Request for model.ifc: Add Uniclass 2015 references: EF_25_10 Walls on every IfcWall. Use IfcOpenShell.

First a look at what the model holds.

```python
import ifcopenshell

model = ifcopenshell.open("model.ifc")
print(model.schema)
print("classifications:", [c.Name for c in model.by_type("IfcClassification")])
for ifc_class in ("IfcDoor", "IfcRoof", "IfcStair", "IfcWall", "IfcWindow"):
    print(ifc_class, len(model.by_type(ifc_class)))
```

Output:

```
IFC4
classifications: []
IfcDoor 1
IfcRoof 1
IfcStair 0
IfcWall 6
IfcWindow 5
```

```python
import ifcopenshell
import ifcopenshell.api.classification

model = ifcopenshell.open("model.ifc")

system = ifcopenshell.api.classification.add_classification(model, classification="Uniclass 2015")

codes = {
    "IfcWall": ("EF_25_10", "Walls"),
}
for ifc_class, (code, name) in codes.items():
    products = model.by_type(ifc_class)
    ifcopenshell.api.classification.add_reference(
        model, products=products, classification=system, identification=code, name=name
    )
    print(code, len(products))

model.write("model_edited.ifc")
```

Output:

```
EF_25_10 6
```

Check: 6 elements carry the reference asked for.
